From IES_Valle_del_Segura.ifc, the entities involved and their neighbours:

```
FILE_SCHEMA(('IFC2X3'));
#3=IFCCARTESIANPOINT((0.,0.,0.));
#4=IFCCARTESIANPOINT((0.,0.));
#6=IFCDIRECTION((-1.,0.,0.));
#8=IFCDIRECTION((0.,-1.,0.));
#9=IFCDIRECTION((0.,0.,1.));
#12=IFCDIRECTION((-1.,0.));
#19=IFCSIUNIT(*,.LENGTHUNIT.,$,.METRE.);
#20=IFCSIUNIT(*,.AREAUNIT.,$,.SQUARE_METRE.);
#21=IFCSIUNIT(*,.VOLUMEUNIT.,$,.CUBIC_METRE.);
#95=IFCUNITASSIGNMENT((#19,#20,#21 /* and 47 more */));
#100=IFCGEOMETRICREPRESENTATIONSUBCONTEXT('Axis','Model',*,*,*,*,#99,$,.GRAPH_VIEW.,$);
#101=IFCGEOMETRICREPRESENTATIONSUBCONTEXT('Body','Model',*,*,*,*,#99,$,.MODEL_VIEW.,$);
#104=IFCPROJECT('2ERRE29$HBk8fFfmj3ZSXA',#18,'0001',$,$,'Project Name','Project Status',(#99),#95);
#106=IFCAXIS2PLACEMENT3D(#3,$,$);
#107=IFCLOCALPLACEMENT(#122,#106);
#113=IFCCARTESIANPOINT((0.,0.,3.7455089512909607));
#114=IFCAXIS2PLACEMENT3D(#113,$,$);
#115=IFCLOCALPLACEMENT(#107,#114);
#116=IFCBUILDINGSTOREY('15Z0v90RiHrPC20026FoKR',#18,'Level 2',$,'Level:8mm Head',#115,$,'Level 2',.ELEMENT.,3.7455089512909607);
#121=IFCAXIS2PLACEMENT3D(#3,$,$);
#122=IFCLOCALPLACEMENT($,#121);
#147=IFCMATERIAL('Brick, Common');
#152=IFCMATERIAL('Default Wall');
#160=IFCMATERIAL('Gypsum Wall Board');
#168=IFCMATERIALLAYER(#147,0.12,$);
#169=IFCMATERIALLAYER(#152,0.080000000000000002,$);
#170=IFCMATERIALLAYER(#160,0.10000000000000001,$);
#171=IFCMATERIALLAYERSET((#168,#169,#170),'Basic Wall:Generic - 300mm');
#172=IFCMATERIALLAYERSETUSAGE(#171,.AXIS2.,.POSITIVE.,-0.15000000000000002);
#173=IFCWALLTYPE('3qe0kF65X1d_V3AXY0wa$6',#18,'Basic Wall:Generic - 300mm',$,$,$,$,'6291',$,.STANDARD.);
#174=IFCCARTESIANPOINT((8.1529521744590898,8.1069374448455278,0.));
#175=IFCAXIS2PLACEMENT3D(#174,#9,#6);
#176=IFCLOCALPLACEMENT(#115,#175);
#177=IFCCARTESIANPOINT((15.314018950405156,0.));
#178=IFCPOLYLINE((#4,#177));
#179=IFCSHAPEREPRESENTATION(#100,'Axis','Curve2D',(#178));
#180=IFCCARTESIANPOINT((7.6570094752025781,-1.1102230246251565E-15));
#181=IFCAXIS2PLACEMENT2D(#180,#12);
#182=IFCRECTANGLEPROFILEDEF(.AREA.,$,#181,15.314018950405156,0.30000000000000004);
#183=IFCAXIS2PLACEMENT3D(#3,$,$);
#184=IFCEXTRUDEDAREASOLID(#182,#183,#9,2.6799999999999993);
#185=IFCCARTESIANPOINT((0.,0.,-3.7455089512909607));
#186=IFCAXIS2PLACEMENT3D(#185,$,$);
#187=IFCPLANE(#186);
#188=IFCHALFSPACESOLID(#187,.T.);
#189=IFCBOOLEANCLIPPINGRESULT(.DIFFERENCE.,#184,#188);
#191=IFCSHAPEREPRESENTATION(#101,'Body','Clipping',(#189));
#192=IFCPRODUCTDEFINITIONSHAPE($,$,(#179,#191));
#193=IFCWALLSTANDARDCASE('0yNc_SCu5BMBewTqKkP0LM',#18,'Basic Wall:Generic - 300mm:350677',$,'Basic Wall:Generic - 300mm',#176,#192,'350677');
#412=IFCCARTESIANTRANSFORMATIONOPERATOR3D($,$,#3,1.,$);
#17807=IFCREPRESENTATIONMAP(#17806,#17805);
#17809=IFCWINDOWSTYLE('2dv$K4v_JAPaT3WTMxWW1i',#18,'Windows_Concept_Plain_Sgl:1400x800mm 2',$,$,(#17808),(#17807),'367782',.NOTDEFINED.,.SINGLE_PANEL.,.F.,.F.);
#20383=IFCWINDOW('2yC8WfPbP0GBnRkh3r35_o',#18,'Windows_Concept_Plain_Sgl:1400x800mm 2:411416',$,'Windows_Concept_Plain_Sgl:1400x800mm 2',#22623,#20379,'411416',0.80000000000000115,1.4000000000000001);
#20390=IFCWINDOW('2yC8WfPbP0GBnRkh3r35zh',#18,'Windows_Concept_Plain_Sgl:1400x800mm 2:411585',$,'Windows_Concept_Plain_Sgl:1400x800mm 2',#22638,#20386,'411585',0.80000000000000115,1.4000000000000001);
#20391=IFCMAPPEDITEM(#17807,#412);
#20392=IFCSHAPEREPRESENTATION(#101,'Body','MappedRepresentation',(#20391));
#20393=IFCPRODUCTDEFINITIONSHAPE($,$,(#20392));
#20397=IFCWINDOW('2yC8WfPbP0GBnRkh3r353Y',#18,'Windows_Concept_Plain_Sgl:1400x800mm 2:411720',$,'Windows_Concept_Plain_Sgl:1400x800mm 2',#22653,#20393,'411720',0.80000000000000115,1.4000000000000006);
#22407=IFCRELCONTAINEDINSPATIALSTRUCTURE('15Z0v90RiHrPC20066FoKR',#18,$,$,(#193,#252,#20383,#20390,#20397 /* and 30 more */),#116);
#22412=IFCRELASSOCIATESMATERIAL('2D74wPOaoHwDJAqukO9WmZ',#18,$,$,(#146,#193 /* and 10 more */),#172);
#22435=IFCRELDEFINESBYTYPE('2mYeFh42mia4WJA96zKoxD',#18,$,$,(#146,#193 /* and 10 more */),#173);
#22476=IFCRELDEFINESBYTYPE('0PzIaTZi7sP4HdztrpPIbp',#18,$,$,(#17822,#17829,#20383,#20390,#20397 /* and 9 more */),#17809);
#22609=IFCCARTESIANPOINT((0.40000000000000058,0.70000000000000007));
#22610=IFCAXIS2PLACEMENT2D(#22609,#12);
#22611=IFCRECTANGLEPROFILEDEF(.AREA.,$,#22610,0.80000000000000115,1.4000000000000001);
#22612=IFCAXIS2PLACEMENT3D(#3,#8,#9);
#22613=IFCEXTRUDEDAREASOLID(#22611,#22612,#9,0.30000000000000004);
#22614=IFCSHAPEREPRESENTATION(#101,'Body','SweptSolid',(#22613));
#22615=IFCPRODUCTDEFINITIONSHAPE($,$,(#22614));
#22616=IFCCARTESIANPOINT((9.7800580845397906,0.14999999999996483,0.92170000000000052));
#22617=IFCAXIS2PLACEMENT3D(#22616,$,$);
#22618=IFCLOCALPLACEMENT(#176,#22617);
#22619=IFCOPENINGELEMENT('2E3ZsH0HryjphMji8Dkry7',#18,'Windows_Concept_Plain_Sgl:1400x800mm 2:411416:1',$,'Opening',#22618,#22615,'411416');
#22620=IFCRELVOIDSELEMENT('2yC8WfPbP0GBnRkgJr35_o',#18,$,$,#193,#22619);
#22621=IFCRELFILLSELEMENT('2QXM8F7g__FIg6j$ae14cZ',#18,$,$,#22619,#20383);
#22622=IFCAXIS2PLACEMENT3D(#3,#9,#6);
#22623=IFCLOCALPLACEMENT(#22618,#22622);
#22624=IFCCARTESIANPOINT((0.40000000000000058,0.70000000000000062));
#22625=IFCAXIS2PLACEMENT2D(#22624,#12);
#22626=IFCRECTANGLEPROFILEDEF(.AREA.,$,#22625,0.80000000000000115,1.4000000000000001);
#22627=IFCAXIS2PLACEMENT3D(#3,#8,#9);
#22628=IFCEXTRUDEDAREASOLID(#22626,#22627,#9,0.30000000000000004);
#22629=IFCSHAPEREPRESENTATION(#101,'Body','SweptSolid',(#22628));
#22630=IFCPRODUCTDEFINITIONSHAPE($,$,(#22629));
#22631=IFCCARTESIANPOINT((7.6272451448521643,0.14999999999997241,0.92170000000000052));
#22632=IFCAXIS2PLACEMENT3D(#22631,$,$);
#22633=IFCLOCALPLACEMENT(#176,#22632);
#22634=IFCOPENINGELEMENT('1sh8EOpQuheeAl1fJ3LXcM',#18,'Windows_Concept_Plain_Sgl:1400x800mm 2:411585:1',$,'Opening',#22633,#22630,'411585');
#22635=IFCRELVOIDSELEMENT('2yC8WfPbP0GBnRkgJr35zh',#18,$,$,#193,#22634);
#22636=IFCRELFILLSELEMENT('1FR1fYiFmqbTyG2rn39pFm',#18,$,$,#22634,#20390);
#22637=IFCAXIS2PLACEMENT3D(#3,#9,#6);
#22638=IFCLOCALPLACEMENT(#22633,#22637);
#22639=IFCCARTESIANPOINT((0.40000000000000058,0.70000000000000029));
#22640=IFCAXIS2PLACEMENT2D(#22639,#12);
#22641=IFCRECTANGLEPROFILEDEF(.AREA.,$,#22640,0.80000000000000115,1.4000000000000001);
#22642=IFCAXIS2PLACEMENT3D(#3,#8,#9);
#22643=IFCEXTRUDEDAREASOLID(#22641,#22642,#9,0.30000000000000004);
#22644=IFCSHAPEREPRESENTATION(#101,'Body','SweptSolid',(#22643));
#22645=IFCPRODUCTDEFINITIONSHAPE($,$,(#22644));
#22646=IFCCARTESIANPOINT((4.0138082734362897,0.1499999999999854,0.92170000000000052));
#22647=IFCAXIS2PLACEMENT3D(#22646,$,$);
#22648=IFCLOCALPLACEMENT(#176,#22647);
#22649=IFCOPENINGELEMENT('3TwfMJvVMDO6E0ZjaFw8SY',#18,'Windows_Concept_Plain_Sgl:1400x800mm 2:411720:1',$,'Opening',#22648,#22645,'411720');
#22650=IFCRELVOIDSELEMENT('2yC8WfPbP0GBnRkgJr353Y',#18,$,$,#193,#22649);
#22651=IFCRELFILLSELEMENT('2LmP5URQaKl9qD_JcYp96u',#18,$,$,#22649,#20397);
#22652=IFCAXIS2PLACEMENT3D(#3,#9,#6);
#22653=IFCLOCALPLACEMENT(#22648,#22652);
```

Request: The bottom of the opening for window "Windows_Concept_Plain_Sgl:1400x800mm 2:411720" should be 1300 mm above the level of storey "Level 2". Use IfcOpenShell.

```python
import numpy as np
import ifcopenshell
import ifcopenshell.api.geometry
import ifcopenshell.geom
import ifcopenshell.util.element
import ifcopenshell.util.placement
import ifcopenshell.util.shape
import ifcopenshell.util.unit

model = ifcopenshell.open("IES_Valle_del_Segura.ifc")
unit_scale = ifcopenshell.util.unit.calculate_unit_scale(model)

window = model.by_id(20397)
opening = window.FillsVoids[0].RelatingOpeningElement
storey = ifcopenshell.util.element.get_container(window, ifc_class="IfcBuildingStorey")
level = ifcopenshell.util.placement.get_local_placement(storey.ObjectPlacement)[2, 3]

# The opening's origin need not be at the sill, so measure its lowest point.
shape = ifcopenshell.geom.create_shape(ifcopenshell.geom.settings(), opening)
bottom = ifcopenshell.util.shape.get_shape_bottom_elevation(shape, shape.geometry) / unit_scale
dz = level + 1.3 / unit_scale - bottom

shift = np.array([0.0, 0.0, dz])
# The window is placed relative to its opening, so it follows when the opening moves.
matrix = ifcopenshell.util.placement.get_local_placement(opening.ObjectPlacement)
matrix[:3, 3] += shift
ifcopenshell.api.geometry.edit_object_placement(
    model, product=opening, matrix=matrix, is_si=False, should_transform_children=True
)

print(f"moved by {dz * unit_scale:+.3f} m")

model.write("IES_Valle_del_Segura_rev.ifc")
```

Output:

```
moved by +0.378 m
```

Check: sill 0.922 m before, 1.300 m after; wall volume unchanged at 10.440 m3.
